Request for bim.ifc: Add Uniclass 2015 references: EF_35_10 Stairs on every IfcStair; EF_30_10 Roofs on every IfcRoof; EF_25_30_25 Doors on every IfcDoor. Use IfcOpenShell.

First a look at what the model holds.

```python
import ifcopenshell

model = ifcopenshell.open("bim.ifc")
print(model.schema)
print("classifications:", [c.Name for c in model.by_type("IfcClassification")])
for ifc_class in ("IfcDoor", "IfcRoof", "IfcStair", "IfcWall", "IfcWindow"):
    print(ifc_class, len(model.by_type(ifc_class)))
```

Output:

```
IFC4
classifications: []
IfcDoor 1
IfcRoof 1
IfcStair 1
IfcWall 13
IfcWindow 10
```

```python
import ifcopenshell
import ifcopenshell.api.classification

model = ifcopenshell.open("bim.ifc")

system = ifcopenshell.api.classification.add_classification(model, classification="Uniclass 2015")

codes = {
    "IfcStair": ("EF_35_10", "Stairs"),
    "IfcRoof": ("EF_30_10", "Roofs"),
    "IfcDoor": ("EF_25_30_25", "Doors"),
}
for ifc_class, (code, name) in codes.items():
    products = model.by_type(ifc_class)
    ifcopenshell.api.classification.add_reference(
        model, products=products, classification=system, identification=code, name=name
    )
    print(code, len(products))

model.write("bim_updated.ifc")
```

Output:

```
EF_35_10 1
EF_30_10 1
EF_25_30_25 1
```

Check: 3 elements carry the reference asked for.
